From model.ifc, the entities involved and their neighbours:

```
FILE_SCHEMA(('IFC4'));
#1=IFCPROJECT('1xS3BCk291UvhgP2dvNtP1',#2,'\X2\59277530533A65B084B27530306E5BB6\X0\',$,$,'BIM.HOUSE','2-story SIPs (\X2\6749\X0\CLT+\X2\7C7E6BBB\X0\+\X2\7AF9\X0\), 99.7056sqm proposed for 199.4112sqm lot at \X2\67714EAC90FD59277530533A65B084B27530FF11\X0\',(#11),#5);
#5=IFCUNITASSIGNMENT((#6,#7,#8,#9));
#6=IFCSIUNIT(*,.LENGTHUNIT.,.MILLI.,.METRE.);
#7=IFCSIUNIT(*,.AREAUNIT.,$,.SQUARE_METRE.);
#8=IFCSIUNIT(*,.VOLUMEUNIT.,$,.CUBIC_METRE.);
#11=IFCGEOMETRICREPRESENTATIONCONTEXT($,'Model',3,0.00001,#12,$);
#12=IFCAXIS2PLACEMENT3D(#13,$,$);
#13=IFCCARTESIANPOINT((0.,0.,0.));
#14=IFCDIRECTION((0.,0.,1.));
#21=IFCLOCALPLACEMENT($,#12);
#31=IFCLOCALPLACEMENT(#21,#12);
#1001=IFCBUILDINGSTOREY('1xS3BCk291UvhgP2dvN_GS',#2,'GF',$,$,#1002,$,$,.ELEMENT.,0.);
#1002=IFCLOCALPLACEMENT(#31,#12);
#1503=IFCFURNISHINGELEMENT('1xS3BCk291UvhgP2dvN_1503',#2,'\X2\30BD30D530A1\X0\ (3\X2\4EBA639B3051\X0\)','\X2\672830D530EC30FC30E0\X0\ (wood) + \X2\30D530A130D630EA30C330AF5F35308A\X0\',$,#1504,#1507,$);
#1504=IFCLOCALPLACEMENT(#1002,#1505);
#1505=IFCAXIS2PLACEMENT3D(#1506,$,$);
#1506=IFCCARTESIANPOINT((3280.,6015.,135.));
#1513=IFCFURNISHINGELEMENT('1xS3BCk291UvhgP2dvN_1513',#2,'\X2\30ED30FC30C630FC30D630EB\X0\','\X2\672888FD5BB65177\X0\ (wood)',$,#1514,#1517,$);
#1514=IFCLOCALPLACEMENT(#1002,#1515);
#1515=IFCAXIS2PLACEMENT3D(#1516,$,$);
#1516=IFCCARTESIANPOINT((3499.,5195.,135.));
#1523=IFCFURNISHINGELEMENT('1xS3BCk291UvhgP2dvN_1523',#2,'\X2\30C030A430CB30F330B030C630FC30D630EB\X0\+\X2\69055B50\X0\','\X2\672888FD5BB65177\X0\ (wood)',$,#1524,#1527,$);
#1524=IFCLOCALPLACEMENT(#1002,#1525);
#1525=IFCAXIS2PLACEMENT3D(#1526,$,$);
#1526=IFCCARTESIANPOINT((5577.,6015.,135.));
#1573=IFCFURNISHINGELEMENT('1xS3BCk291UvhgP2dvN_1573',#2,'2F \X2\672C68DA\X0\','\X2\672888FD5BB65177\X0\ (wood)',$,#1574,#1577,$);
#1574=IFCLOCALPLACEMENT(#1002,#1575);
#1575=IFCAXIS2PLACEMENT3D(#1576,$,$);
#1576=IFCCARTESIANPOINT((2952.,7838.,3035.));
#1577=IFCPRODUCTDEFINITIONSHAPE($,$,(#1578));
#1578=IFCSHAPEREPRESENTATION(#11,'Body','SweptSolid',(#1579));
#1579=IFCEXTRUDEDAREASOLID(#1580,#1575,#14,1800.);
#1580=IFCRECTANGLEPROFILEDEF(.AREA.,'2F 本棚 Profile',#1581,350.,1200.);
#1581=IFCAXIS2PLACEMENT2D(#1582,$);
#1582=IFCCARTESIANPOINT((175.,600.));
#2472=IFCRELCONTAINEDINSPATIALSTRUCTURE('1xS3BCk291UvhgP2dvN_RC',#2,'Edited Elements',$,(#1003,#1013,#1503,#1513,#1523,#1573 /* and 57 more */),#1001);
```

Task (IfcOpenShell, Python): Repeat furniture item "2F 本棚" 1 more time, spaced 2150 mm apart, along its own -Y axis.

```python
import ifcopenshell
import ifcopenshell.api.geometry
import ifcopenshell.api.root
import ifcopenshell.util.element
import ifcopenshell.util.placement
import ifcopenshell.util.unit

model = ifcopenshell.open("model.ifc")
unit_scale = ifcopenshell.util.unit.calculate_unit_scale(model)


def reuse_history(source, copy):
    """copy_class also copies each property set's owner history, people and application; keep the originals."""
    for rel in copy.IsDefinedBy:
        if rel.is_a("IfcRelDefinesByProperties") and (history := rel.RelatingPropertyDefinition.OwnerHistory):
            rel.RelatingPropertyDefinition.OwnerHistory = source.OwnerHistory
            ifcopenshell.util.element.remove_deep2(model, history)


source = model.by_guid("1xS3BCk291UvhgP2dvN_1573")
base = ifcopenshell.util.placement.get_local_placement(source.ObjectPlacement)
step = -base[:3, 1] * 2.15 / unit_scale

for i in range(1, 2):
    copy = ifcopenshell.api.root.copy_class(model, product=source)
    copy.Representation = ifcopenshell.util.element.copy_deep(
        model, source.Representation, exclude=["IfcGeometricRepresentationContext", "IfcRepresentationMap"]
    )
    reuse_history(source, copy)
    matrix = base.copy()
    matrix[:3, 3] += i * step
    print("added at", matrix[:3, 3].round(3) + 0.0)
    ifcopenshell.api.geometry.edit_object_placement(model, product=copy, matrix=matrix, is_si=False)

model.write("model_updated.ifc")
```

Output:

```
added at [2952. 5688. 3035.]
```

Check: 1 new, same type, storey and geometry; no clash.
